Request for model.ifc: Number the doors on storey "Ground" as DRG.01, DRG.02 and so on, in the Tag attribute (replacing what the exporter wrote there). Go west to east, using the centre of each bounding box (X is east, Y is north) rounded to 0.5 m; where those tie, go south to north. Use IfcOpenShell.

First a look at what the model holds.

```python
import ifcopenshell
import ifcopenshell.util.element
import ifcopenshell.util.placement

model = ifcopenshell.open("model.ifc")
print(model.schema)
storey = next(s for s in model.by_type("IfcBuildingStorey") if s.Name == "Ground")
doors = [e for e in ifcopenshell.util.element.get_decomposition(storey) if e.is_a("IfcDoor")]
for e in sorted(doors, key=lambda e: e.id()):
    origin = ifcopenshell.util.placement.get_local_placement(e.ObjectPlacement)[:3, 3]
    print(e.id(), e.Tag, e.Name, origin.round(2) + 0.0, sep=" | ")
```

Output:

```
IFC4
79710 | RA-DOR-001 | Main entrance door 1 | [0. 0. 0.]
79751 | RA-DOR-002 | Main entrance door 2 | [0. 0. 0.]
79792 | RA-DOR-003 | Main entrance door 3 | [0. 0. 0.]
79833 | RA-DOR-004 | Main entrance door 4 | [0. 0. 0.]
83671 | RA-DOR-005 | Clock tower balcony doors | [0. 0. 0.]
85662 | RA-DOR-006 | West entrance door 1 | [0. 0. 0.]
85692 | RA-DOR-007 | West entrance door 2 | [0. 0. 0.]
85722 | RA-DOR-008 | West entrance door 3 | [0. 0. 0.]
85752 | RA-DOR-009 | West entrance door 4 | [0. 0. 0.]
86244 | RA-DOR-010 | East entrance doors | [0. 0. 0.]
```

```python
import ifcopenshell
import ifcopenshell.geom
import ifcopenshell.util.element
import ifcopenshell.util.shape

model = ifcopenshell.open("model.ifc")
settings = ifcopenshell.geom.settings()
settings.set("use-world-coords", True)


def centre(element):
    shape = ifcopenshell.geom.create_shape(settings, element)
    return ifcopenshell.util.shape.get_bbox_centroid(shape.geometry)


storey = next(s for s in model.by_type("IfcBuildingStorey") if s.Name == "Ground")
doors = [e for e in ifcopenshell.util.element.get_decomposition(storey) if e.is_a("IfcDoor")]

# Insertion points can sit at a corner or the storey origin, so sort by the geometry (in metres).
centres = {e: centre(e) for e in doors}
doors.sort(key=lambda e: (round(centres[e][0] / 0.5), centres[e][1]))

for i, e in enumerate(doors, start=1):
    number = f"DRG.{i:02d}"
    e.Tag = number
    print(e.id(), number)

model.write("model_rev.ifc")
```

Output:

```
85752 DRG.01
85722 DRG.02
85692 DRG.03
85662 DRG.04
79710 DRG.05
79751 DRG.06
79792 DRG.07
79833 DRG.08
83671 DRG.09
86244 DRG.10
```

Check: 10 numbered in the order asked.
